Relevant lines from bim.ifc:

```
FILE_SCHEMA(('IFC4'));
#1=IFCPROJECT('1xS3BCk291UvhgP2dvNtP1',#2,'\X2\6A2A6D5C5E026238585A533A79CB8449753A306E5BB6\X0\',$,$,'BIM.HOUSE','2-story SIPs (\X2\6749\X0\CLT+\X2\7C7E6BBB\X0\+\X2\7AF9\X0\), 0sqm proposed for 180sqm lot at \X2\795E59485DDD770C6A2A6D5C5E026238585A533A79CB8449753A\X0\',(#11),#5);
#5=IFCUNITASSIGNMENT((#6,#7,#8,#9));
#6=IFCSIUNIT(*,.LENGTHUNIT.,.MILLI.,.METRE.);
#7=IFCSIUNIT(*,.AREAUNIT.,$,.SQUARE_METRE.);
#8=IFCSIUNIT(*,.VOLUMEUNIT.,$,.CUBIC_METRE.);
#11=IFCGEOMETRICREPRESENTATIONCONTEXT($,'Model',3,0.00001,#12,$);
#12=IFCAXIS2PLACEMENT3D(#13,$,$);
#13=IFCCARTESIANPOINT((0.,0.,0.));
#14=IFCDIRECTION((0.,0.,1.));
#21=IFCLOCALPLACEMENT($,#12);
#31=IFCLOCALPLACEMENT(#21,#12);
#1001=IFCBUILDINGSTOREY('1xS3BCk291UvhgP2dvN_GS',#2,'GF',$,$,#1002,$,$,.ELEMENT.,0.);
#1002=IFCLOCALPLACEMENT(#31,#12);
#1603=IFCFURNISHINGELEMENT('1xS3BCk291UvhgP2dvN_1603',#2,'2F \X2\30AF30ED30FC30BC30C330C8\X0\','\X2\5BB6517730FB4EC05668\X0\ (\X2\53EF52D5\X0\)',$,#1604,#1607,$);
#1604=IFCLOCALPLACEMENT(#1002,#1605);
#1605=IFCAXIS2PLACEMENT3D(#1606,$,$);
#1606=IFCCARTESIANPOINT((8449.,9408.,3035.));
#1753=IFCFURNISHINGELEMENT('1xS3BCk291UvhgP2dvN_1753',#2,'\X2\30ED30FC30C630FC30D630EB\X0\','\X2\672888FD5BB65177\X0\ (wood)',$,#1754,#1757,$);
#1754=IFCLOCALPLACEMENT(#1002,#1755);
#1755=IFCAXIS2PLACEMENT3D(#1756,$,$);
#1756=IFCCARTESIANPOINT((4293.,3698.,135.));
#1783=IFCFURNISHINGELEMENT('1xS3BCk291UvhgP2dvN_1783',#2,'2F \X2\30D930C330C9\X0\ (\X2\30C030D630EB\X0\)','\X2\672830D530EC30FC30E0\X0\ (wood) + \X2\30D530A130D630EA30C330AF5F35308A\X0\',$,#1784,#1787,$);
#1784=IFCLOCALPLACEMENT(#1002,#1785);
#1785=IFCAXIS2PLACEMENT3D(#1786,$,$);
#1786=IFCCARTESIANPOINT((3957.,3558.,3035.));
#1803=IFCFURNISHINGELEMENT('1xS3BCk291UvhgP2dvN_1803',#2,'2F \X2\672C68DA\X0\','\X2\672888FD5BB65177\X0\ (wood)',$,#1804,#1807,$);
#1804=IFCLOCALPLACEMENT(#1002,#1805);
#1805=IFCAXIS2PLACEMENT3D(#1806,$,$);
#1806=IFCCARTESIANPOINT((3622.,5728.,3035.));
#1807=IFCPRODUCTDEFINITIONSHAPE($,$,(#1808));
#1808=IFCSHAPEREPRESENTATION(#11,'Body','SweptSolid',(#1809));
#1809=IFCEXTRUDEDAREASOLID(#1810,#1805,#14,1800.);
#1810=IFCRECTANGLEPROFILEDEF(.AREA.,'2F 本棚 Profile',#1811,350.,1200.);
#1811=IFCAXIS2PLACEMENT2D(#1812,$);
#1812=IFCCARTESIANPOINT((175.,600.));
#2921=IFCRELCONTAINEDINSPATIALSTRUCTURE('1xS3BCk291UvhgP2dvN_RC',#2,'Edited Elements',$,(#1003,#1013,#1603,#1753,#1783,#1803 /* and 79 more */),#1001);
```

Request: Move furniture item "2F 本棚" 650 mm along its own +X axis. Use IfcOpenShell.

```python
import ifcopenshell
import ifcopenshell.api.geometry
import ifcopenshell.util.placement

model = ifcopenshell.open("bim.ifc")

item = model.by_guid("1xS3BCk291UvhgP2dvN_1803")
matrix = ifcopenshell.util.placement.get_local_placement(item.ObjectPlacement)
matrix[:3, 3] += matrix[:3, 0] * 650.0
ifcopenshell.api.geometry.edit_object_placement(model, product=item, matrix=matrix, is_si=False)

print(ifcopenshell.util.placement.get_local_placement(item.ObjectPlacement).round(3) + 0.0)

model.write("bim_updated.ifc")
```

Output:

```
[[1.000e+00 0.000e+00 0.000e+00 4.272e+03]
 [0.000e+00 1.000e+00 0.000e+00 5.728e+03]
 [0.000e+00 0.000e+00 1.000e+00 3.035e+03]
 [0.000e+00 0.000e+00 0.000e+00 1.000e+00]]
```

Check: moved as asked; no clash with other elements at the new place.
